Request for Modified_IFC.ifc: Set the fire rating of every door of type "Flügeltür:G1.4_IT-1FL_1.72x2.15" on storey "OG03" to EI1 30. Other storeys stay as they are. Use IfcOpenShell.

First a look at what the model holds.

```python
import ifcopenshell
import ifcopenshell.util.element

model = ifcopenshell.open("Modified_IFC.ifc")
print(model.schema)
storey = next(s for s in model.by_type("IfcBuildingStorey") if s.Name == "OG03")
doors = [e for e in ifcopenshell.util.element.get_decomposition(storey) if e.is_a("IfcDoor")]
seen = {}
for e in doors:
    element_type = ifcopenshell.util.element.get_type(e)
    key = (element_type.Name if element_type != e and element_type else None, ifcopenshell.util.element.get_pset(e, "Pset_DoorCommon", "FireRating"))
    seen[key] = seen.get(key, 0) + 1
for (name, value), count in sorted(seen.items(), key=str):
    print(count, "x", name, "|", value)
```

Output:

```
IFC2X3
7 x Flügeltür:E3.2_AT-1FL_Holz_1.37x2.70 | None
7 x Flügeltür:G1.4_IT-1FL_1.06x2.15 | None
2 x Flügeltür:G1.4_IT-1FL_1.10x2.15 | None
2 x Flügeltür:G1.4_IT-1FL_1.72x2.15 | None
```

```python
import ifcopenshell
import ifcopenshell.api.pset
import ifcopenshell.util.element

model = ifcopenshell.open("Modified_IFC.ifc")

storey = next(s for s in model.by_type("IfcBuildingStorey") if s.Name == "OG03")
doors = [e for e in ifcopenshell.util.element.get_decomposition(storey) if e.is_a("IfcDoor")]

count = 0
for e in doors:
    element_type = ifcopenshell.util.element.get_type(e)
    if element_type in (None, e) or element_type.Name != "Flügeltür:G1.4_IT-1FL_1.72x2.15":
        continue
    # add_pset returns the element's existing set when there is one.
    pset = ifcopenshell.api.pset.add_pset(model, product=e, name="Pset_DoorCommon")
    ifcopenshell.api.pset.edit_pset(model, pset=pset, properties={"FireRating": "EI1 30"})
    count += 1

print(count, "doors updated")

model.write("Modified_IFC_updated.ifc")
```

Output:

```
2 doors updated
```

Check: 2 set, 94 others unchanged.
